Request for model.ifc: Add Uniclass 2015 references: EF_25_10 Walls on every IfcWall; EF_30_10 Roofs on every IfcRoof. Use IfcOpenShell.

First a look at what the model holds.

```python
import ifcopenshell

model = ifcopenshell.open("model.ifc")
print(model.schema)
print("classifications:", [c.Name for c in model.by_type("IfcClassification")])
for ifc_class in ("IfcDoor", "IfcRoof", "IfcStair", "IfcWall", "IfcWindow"):
    print(ifc_class, len(model.by_type(ifc_class)))
```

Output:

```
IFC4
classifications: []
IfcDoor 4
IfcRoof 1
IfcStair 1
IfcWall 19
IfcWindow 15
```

```python
import ifcopenshell
import ifcopenshell.api.classification

model = ifcopenshell.open("model.ifc")

system = ifcopenshell.api.classification.add_classification(model, classification="Uniclass 2015")

codes = {
    "IfcWall": ("EF_25_10", "Walls"),
    "IfcRoof": ("EF_30_10", "Roofs"),
}
for ifc_class, (code, name) in codes.items():
    products = model.by_type(ifc_class)
    ifcopenshell.api.classification.add_reference(
        model, products=products, classification=system, identification=code, name=name
    )
    print(code, len(products))

model.write("model_edited.ifc")
```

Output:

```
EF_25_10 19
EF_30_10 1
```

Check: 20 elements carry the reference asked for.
